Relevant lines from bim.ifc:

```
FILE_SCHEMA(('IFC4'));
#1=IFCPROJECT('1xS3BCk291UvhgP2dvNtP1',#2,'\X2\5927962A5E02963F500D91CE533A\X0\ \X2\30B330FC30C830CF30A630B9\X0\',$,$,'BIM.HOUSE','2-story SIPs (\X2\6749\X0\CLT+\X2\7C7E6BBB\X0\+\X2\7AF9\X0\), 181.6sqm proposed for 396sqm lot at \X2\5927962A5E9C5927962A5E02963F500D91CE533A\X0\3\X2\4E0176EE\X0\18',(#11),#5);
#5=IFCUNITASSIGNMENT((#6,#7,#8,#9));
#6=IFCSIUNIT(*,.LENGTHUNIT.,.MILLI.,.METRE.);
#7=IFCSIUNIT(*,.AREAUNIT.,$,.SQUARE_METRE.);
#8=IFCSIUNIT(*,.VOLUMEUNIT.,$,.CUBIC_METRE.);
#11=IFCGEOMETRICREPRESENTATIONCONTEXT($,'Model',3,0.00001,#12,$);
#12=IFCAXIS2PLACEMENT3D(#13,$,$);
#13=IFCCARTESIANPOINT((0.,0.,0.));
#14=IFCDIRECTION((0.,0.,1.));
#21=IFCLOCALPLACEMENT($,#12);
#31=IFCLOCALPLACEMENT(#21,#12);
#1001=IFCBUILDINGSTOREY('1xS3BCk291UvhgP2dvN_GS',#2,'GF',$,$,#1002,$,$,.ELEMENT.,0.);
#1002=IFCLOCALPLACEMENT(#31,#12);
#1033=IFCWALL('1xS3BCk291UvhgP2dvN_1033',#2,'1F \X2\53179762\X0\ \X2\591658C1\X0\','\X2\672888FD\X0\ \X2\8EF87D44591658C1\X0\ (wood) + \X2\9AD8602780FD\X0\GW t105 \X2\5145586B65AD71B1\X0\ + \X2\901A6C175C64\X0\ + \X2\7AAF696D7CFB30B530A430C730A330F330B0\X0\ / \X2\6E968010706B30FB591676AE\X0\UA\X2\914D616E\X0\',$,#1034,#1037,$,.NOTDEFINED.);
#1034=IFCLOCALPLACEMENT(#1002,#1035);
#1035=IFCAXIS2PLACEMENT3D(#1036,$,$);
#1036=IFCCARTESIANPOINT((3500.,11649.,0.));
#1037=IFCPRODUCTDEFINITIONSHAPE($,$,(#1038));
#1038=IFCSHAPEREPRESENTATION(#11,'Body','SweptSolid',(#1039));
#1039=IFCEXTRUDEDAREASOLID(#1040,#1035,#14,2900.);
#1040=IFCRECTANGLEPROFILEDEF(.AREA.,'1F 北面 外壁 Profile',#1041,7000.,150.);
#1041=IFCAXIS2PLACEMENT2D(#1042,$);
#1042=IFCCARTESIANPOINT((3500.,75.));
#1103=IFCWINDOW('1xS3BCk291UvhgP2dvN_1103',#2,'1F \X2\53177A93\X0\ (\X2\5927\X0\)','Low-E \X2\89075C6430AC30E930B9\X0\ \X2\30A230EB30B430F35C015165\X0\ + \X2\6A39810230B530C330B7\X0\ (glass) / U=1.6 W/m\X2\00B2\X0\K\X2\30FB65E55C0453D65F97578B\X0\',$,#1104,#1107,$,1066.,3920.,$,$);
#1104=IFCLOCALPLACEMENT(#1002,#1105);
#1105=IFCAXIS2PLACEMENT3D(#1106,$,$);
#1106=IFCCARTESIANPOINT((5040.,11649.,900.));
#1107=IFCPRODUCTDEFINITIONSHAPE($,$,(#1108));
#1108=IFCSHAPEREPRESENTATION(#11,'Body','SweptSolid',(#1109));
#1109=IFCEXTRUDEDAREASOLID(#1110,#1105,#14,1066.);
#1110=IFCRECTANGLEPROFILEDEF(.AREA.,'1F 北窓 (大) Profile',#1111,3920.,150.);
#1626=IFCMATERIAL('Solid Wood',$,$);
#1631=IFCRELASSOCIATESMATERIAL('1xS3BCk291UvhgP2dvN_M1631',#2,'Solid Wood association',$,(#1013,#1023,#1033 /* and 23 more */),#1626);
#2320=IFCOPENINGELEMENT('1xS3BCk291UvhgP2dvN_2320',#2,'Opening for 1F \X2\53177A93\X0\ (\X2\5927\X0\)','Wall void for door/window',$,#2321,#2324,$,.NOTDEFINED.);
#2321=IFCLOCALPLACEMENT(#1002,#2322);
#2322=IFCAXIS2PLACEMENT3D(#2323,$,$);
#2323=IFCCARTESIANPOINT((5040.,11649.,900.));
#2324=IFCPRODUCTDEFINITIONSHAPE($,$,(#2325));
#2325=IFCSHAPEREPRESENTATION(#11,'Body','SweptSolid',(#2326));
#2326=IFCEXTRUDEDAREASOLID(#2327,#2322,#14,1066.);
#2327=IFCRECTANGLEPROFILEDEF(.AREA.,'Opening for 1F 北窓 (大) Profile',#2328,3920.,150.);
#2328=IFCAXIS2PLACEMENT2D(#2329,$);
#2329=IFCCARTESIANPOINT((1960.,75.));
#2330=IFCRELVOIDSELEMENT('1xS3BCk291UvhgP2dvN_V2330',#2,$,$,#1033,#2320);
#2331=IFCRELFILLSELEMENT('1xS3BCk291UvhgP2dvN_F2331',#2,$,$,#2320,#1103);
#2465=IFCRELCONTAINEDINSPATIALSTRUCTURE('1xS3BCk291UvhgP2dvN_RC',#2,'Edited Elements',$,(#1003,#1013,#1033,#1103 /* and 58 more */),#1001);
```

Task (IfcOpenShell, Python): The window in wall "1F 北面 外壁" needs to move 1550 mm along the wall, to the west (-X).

```python
import ifcopenshell
import ifcopenshell.api.geometry
import ifcopenshell.util.placement
import ifcopenshell.util.unit

model = ifcopenshell.open("bim.ifc")
unit_scale = ifcopenshell.util.unit.calculate_unit_scale(model)

window = model.by_id(1103)
opening = window.FillsVoids[0].RelatingOpeningElement
wall = opening.VoidsElements[0].RelatingBuildingElement

wall_matrix = ifcopenshell.util.placement.get_local_placement(wall.ObjectPlacement)
shift = wall_matrix[:3, 0] * -1.55 / unit_scale
before = ifcopenshell.util.placement.get_local_placement(window.ObjectPlacement)[:3, 3].copy()

# The window is not placed relative to its opening, so move both.
for product in (opening, window):
    matrix = ifcopenshell.util.placement.get_local_placement(product.ObjectPlacement)
    matrix[:3, 3] += shift
    ifcopenshell.api.geometry.edit_object_placement(model, product=product, matrix=matrix, is_si=False)

after = ifcopenshell.util.placement.get_local_placement(window.ObjectPlacement)[:3, 3]
print("window moved by", (after - before).round(3) + 0.0)

model.write("bim_rev.ifc")
```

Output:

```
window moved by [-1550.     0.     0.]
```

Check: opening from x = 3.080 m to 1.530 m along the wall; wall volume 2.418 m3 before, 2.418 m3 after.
